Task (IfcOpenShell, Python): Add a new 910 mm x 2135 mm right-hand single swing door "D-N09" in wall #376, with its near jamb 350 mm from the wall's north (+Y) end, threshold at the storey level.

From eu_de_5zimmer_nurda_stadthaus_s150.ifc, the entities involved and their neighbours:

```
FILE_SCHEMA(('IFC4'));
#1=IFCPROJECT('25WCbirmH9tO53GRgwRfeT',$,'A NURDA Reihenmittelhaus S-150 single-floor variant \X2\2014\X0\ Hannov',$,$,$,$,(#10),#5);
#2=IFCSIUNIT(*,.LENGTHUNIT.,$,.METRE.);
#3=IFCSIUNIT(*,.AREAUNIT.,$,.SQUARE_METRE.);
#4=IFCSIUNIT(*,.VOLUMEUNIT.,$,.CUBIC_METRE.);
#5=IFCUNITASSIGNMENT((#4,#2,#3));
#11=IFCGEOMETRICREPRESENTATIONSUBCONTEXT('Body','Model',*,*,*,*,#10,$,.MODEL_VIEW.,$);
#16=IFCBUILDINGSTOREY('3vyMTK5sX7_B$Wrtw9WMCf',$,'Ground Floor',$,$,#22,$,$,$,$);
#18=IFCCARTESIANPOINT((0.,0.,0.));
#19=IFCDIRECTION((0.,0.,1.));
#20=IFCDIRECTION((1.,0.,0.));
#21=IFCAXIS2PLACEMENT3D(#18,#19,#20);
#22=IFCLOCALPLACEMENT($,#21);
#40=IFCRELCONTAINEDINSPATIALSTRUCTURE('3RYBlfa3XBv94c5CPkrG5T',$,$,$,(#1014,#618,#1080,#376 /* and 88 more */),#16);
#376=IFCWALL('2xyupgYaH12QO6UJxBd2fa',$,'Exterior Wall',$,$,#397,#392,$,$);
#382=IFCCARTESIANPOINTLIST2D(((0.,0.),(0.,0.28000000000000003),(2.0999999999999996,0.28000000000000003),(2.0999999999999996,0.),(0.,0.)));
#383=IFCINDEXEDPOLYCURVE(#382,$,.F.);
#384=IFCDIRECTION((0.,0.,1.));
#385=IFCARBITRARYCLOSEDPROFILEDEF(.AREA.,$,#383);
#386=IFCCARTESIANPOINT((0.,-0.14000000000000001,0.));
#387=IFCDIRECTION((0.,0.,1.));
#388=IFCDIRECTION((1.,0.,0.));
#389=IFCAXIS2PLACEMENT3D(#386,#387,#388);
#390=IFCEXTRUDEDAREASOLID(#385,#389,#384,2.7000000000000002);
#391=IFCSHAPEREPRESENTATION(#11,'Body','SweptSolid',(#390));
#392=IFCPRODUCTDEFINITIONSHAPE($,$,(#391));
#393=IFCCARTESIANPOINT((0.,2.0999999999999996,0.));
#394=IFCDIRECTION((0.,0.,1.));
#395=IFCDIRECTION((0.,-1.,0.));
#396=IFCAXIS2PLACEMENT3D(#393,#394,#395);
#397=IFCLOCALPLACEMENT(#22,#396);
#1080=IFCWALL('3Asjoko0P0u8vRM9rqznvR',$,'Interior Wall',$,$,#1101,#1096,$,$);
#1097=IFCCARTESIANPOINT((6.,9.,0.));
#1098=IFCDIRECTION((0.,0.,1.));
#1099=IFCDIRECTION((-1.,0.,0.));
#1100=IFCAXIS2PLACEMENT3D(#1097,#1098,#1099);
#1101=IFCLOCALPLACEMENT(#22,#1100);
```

```python
import numpy as np
import ifcopenshell
import ifcopenshell.api.feature
import ifcopenshell.api.geometry
import ifcopenshell.api.root
import ifcopenshell.api.spatial
import ifcopenshell.geom
import ifcopenshell.util.element
import ifcopenshell.util.placement
import ifcopenshell.util.representation
import ifcopenshell.util.shape
import ifcopenshell.util.unit

model = ifcopenshell.open("eu_de_5zimmer_nurda_stadthaus_s150.ifc")
unit_scale = ifcopenshell.util.unit.calculate_unit_scale(model)
settings = ifcopenshell.geom.settings()


def volume(element):
    """Net volume in cubic metres, openings subtracted."""
    shape = ifcopenshell.geom.create_shape(settings, element)
    return ifcopenshell.util.shape.get_volume(shape.geometry)


wall = model.by_id(376)
storey = ifcopenshell.util.element.get_container(wall, ifc_class="IfcBuildingStorey")
context = ifcopenshell.util.representation.get_context(model, "Model", "Body", "MODEL_VIEW")
before = volume(wall)

width, height, from_end, sill = 0.91, 2.135, 0.35, 0.0  # metres

# The wall runs along its own X axis, and the end named is its -X end.
wall_shape = ifcopenshell.geom.create_shape(settings, wall)
x, y, z = ifcopenshell.util.shape.get_vertices(wall_shape.geometry).T
start = x.min() + from_end
face, thickness = float(y.min()), float(y.max() - y.min())
wall_matrix = ifcopenshell.util.placement.get_local_placement(wall.ObjectPlacement)
level = ifcopenshell.util.placement.get_local_placement(storey.ObjectPlacement)[2, 3]


def in_wall(x, y):
    """Placement at x, y metres in the wall's axes, at sill height."""
    matrix = wall_matrix.copy()
    matrix[:, 3] = wall_matrix @ np.array([x / unit_scale, y / unit_scale, 0.0, 1.0])
    matrix[2, 3] = level + sill / unit_scale
    return matrix


# Opening: a box that overshoots both wall faces by 50 mm.
opening = ifcopenshell.api.root.create_entity(model, ifc_class="IfcOpeningElement", predefined_type="OPENING")
box = ifcopenshell.api.geometry.add_wall_representation(
    model, context=context, length=width, height=height, thickness=thickness + 0.1
)
ifcopenshell.api.geometry.assign_representation(model, product=opening, representation=box)
ifcopenshell.api.geometry.edit_object_placement(model, product=opening, matrix=in_wall(start, face - 0.05), is_si=False)
ifcopenshell.api.feature.add_feature(model, feature=opening, element=wall)

door = ifcopenshell.api.root.create_entity(model, ifc_class="IfcDoor", name="D-N09", predefined_type="DOOR")
door.OverallWidth, door.OverallHeight = width / unit_scale, height / unit_scale
door.OperationType = "SINGLE_SWING_RIGHT"
body = ifcopenshell.api.geometry.add_door_representation(
    model,
    context=context,
    overall_width=door.OverallWidth,
    overall_height=door.OverallHeight,
    operation_type="SINGLE_SWING_RIGHT",
    lining_properties={"LiningDepth": thickness / unit_scale, "ThresholdDepth": thickness / unit_scale},
)
ifcopenshell.api.geometry.assign_representation(model, product=door, representation=body)
ifcopenshell.api.spatial.assign_container(model, products=[door], relating_structure=storey)
ifcopenshell.api.feature.add_filling(model, opening=opening, element=door)

# The lining spans the wall, so the door starts at the wall face.
ifcopenshell.api.geometry.edit_object_placement(model, product=door, matrix=in_wall(start, face), is_si=False)

after = volume(wall)

print(f"wall volume {before:.3f} -> {after:.3f} m3")

model.write("eu_de_5zimmer_nurda_stadthaus_s150_edited.ifc")
```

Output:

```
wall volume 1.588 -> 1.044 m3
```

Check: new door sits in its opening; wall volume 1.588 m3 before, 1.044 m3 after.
